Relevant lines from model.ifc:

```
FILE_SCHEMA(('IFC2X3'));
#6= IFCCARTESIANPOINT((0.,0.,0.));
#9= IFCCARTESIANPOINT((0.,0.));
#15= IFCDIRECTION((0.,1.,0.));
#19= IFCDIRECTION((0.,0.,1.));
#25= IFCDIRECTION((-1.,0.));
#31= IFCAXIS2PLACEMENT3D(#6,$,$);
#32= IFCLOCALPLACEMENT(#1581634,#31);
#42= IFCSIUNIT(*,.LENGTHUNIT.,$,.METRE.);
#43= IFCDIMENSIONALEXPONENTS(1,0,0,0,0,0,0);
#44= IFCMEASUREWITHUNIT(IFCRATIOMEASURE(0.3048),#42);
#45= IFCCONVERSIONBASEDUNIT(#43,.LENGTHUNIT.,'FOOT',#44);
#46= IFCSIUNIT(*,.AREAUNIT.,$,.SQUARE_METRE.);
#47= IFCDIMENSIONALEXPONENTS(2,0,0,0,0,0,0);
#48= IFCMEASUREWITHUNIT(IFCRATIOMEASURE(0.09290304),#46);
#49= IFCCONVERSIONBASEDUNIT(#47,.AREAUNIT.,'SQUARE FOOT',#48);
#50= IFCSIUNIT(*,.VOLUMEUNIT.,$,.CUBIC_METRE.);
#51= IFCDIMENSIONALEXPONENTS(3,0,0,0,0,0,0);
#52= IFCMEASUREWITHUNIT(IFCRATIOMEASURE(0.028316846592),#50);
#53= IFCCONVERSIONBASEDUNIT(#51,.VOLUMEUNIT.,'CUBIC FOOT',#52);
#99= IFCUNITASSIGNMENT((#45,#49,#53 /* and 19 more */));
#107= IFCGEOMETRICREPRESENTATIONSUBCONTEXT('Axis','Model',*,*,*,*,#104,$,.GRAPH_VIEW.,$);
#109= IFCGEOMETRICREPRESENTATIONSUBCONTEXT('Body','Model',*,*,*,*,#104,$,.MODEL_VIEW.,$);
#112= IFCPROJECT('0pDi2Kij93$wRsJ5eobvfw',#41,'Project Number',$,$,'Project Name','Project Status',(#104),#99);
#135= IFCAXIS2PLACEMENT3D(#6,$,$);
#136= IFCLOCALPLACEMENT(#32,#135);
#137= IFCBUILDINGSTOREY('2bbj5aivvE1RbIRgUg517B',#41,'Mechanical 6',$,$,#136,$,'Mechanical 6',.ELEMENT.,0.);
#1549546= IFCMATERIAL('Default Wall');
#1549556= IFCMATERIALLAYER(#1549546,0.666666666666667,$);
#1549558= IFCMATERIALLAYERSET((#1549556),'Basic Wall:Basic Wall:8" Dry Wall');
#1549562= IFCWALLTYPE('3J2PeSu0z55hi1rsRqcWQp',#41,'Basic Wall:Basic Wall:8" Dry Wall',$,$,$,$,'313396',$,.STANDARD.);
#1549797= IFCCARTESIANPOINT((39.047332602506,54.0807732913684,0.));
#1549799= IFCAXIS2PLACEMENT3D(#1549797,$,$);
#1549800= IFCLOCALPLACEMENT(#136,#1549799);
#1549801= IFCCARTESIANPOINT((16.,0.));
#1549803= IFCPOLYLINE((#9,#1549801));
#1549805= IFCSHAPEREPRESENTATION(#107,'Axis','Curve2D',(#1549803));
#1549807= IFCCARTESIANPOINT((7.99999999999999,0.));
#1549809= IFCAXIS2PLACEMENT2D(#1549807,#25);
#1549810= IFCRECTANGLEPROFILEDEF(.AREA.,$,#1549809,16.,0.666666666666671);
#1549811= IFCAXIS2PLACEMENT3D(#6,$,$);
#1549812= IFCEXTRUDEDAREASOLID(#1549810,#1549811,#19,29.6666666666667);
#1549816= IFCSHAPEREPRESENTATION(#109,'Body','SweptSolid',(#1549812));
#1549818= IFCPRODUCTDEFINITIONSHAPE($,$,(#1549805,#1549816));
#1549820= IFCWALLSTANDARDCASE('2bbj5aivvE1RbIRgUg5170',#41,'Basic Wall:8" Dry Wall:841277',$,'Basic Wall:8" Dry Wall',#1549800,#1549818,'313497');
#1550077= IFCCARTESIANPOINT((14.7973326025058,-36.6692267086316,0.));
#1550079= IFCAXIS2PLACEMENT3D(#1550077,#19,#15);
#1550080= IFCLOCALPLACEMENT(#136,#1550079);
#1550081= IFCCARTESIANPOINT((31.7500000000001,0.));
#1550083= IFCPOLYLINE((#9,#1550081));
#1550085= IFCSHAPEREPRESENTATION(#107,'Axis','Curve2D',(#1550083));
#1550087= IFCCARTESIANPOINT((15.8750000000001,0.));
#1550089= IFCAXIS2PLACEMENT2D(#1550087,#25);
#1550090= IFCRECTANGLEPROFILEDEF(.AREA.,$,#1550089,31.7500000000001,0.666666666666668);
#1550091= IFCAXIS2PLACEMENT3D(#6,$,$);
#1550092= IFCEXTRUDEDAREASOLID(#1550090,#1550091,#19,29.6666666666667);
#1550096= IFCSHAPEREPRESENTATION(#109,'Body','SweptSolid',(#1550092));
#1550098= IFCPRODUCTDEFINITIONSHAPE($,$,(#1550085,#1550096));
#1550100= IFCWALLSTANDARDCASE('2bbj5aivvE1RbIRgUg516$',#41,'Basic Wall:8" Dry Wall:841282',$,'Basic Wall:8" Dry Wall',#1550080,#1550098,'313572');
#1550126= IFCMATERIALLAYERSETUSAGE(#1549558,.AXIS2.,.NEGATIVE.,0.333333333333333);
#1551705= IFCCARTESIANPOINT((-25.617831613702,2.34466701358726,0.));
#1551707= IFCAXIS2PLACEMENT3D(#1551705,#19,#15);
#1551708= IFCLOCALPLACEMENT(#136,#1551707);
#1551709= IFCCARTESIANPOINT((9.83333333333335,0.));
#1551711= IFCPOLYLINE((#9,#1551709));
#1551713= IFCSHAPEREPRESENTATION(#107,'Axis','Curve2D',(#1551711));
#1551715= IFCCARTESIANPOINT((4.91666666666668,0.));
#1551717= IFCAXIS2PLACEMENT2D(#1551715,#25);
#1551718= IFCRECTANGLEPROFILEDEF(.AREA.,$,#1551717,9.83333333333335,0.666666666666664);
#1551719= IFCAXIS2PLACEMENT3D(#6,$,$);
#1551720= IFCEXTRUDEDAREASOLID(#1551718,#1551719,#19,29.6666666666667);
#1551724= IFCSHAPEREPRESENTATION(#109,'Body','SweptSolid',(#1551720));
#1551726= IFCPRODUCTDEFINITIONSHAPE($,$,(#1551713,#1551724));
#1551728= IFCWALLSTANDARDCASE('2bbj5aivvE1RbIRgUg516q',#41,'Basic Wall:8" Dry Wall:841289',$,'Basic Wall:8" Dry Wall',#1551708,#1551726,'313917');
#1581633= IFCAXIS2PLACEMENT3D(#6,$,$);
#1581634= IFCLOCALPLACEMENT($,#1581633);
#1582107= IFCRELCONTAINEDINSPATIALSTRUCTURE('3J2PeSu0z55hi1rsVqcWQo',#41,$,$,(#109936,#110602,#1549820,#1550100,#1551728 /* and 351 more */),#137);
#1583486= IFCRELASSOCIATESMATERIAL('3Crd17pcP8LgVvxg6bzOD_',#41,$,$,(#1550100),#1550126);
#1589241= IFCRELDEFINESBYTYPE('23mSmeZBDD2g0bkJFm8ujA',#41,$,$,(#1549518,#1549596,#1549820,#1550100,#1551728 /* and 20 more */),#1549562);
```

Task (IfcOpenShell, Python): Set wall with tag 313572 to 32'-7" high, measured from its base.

```python
import ifcopenshell
import ifcopenshell.geom
import ifcopenshell.util.representation
import ifcopenshell.util.shape
import ifcopenshell.util.unit

model = ifcopenshell.open("model.ifc")
unit_scale = ifcopenshell.util.unit.calculate_unit_scale(model)
settings = ifcopenshell.geom.settings()


def volume(element):
    """Net volume in cubic metres, openings subtracted."""
    shape = ifcopenshell.geom.create_shape(settings, element)
    return ifcopenshell.util.shape.get_volume(shape.geometry)


wall = model.by_id(1550100)
before = volume(wall)

body = ifcopenshell.util.representation.get_representation(wall, "Model", "Body")
solid = body.Items[0]
old_height = solid.Depth
solid.Depth = 391 * 0.0254 / unit_scale
after = volume(wall)

print(f"height {old_height:g} -> {solid.Depth:g}, volume {before:.3f} -> {after:.3f} m3")

model.write("model_updated.ifc")
```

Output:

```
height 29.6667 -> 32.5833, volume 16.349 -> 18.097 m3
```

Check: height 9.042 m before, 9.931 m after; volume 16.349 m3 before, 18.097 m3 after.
